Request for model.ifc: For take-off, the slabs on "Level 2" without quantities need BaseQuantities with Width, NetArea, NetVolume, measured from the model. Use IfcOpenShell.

First a look at what the model holds.

```python
import ifcopenshell
import ifcopenshell.util.element
import ifcopenshell.util.unit

model = ifcopenshell.open("model.ifc")
print(model.schema)
for unit_type in ("LENGTHUNIT", "AREAUNIT", "VOLUMEUNIT"):
    print(unit_type, ifcopenshell.util.unit.calculate_unit_scale(model, unit_type))
storey = next(s for s in model.by_type("IfcBuildingStorey") if s.Name == "Level 2")
slabs = [e for e in ifcopenshell.util.element.get_decomposition(storey) if e.is_a("IfcSlab")]
for e in sorted(slabs, key=lambda e: e.id()):
    print(e.id(), e.is_a(), e.Name, list(ifcopenshell.util.element.get_psets(e, qtos_only=True)), sep=" | ")
```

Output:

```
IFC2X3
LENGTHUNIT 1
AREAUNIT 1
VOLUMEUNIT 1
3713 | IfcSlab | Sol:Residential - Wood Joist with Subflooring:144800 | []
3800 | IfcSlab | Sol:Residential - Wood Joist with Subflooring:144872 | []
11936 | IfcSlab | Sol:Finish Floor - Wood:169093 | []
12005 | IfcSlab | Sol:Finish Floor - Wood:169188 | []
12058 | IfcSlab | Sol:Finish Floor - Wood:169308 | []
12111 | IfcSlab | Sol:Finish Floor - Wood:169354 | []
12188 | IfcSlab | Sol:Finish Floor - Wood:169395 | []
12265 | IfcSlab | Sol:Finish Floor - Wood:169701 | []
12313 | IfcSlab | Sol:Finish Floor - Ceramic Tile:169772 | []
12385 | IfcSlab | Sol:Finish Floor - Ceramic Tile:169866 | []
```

```python
import ifcopenshell
import ifcopenshell.api.pset
import ifcopenshell.geom
import ifcopenshell.util.element
import ifcopenshell.util.shape
import ifcopenshell.util.unit

model = ifcopenshell.open("model.ifc")
unit_scale = ifcopenshell.util.unit.calculate_unit_scale(model)
area_scale = ifcopenshell.util.unit.calculate_unit_scale(model, "AREAUNIT")
volume_scale = ifcopenshell.util.unit.calculate_unit_scale(model, "VOLUMEUNIT")
settings = ifcopenshell.geom.settings()

storey = next(s for s in model.by_type("IfcBuildingStorey") if s.Name == "Level 2")
slabs = [e for e in ifcopenshell.util.element.get_decomposition(storey) if e.is_a("IfcSlab")]

for e in sorted(slabs, key=lambda e: e.id()):
    if ifcopenshell.util.element.get_psets(e, qtos_only=True, should_inherit=False):
        continue
    # Geometry comes back in metres, in the element's own axes.
    shape = ifcopenshell.geom.create_shape(settings, e)
    values = {
        "Width": ifcopenshell.util.shape.get_z(shape.geometry) / unit_scale,
        "NetArea": ifcopenshell.util.shape.get_footprint_area(shape.geometry) / area_scale,
        "NetVolume": ifcopenshell.util.shape.get_volume(shape.geometry) / volume_scale,
    }
    qto = ifcopenshell.api.pset.add_qto(model, product=e, name="BaseQuantities")
    ifcopenshell.api.pset.edit_qto(model, qto=qto, properties=values)
    print(e.id(), {k: round(v, 3) for k, v in values.items()})

model.write("model_updated.ifc")
```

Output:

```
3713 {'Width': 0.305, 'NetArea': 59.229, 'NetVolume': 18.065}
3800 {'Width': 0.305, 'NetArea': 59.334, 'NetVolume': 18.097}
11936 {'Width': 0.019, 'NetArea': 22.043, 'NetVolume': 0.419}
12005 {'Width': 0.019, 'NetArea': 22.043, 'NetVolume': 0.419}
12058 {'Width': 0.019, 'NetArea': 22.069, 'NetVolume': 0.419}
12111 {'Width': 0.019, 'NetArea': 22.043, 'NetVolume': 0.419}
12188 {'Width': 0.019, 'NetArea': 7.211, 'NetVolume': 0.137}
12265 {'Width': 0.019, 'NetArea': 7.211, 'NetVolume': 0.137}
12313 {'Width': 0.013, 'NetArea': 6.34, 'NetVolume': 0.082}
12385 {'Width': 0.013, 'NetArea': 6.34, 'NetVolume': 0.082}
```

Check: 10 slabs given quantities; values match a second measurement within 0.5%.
